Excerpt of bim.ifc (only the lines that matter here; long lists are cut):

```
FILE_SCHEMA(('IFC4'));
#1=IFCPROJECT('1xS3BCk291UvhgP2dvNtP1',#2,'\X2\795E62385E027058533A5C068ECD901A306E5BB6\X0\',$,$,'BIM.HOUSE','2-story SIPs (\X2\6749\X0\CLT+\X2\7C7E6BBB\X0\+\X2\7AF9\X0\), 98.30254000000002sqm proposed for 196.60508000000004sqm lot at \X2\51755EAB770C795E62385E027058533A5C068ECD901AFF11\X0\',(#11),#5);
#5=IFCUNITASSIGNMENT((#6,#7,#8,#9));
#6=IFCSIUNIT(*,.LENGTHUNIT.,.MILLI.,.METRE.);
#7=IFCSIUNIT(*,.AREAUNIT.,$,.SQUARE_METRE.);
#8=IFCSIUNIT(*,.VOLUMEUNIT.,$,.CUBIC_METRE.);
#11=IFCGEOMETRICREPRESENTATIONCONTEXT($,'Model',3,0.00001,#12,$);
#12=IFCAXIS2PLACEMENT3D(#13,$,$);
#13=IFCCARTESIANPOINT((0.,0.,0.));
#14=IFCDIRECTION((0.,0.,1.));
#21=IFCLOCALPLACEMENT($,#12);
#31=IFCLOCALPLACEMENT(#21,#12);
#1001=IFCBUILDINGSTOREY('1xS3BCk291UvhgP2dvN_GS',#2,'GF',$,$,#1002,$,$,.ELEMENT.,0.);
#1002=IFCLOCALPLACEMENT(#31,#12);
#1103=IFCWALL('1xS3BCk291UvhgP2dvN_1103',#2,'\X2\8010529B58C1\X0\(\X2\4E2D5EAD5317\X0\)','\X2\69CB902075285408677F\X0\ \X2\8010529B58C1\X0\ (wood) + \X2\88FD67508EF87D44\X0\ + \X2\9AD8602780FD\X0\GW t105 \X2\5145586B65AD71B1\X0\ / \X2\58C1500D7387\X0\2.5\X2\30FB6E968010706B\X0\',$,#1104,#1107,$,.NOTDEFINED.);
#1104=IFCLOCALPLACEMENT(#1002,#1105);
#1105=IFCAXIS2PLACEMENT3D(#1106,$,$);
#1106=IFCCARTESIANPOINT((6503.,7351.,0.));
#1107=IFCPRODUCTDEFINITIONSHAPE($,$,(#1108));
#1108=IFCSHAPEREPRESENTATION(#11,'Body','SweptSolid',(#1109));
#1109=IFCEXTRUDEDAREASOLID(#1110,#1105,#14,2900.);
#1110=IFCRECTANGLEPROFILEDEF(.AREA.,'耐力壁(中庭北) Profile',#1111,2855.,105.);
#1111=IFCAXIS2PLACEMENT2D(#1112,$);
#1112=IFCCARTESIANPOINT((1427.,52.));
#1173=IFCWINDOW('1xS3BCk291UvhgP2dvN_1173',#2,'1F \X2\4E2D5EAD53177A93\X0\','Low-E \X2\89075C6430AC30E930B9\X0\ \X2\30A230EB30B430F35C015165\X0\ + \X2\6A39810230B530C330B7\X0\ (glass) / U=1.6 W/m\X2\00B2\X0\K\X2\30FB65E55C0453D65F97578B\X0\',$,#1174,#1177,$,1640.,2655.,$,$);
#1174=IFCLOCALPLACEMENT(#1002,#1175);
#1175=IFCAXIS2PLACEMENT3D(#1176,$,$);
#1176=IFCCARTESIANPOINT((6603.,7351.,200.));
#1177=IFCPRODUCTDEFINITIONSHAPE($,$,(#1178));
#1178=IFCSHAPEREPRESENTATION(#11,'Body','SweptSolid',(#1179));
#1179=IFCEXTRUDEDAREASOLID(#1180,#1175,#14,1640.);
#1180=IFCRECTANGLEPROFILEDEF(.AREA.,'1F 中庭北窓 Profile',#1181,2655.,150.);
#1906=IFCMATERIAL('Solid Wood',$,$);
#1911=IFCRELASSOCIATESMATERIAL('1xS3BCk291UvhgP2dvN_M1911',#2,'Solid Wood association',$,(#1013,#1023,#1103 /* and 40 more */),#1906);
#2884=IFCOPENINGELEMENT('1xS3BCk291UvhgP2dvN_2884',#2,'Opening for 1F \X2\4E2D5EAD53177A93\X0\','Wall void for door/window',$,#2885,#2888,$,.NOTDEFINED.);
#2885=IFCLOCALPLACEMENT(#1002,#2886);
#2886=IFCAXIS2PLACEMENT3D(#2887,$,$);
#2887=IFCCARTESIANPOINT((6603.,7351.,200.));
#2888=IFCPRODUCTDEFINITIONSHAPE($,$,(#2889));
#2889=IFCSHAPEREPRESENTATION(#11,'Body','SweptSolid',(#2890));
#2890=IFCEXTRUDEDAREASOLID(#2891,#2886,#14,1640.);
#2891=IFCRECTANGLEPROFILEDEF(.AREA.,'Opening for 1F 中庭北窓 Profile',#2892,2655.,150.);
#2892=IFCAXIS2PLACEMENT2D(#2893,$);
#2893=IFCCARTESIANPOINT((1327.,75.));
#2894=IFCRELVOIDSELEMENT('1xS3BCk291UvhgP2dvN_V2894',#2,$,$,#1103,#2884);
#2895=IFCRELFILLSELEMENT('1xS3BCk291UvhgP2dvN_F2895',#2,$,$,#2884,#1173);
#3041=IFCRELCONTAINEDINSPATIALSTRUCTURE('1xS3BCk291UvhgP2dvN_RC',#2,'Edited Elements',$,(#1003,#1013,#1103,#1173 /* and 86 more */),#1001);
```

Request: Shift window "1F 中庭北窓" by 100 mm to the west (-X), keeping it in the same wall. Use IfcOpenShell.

```python
import ifcopenshell
import ifcopenshell.api.geometry
import ifcopenshell.util.placement

model = ifcopenshell.open("bim.ifc")

window = model.by_guid("1xS3BCk291UvhgP2dvN_1173")
opening = window.FillsVoids[0].RelatingOpeningElement
wall = opening.VoidsElements[0].RelatingBuildingElement

wall_matrix = ifcopenshell.util.placement.get_local_placement(wall.ObjectPlacement)
shift = wall_matrix[:3, 0] * -100.0
before = ifcopenshell.util.placement.get_local_placement(window.ObjectPlacement)[:3, 3].copy()

# The window is not placed relative to its opening, so move both.
for product in (opening, window):
    matrix = ifcopenshell.util.placement.get_local_placement(product.ObjectPlacement)
    matrix[:3, 3] += shift
    ifcopenshell.api.geometry.edit_object_placement(model, product=product, matrix=matrix, is_si=False)

after = ifcopenshell.util.placement.get_local_placement(window.ObjectPlacement)[:3, 3]
print("window moved by", (after - before).round(3) + 0.0)

model.write("bim_edited.ifc")
```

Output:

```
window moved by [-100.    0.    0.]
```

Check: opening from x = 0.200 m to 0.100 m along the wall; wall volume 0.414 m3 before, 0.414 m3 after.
